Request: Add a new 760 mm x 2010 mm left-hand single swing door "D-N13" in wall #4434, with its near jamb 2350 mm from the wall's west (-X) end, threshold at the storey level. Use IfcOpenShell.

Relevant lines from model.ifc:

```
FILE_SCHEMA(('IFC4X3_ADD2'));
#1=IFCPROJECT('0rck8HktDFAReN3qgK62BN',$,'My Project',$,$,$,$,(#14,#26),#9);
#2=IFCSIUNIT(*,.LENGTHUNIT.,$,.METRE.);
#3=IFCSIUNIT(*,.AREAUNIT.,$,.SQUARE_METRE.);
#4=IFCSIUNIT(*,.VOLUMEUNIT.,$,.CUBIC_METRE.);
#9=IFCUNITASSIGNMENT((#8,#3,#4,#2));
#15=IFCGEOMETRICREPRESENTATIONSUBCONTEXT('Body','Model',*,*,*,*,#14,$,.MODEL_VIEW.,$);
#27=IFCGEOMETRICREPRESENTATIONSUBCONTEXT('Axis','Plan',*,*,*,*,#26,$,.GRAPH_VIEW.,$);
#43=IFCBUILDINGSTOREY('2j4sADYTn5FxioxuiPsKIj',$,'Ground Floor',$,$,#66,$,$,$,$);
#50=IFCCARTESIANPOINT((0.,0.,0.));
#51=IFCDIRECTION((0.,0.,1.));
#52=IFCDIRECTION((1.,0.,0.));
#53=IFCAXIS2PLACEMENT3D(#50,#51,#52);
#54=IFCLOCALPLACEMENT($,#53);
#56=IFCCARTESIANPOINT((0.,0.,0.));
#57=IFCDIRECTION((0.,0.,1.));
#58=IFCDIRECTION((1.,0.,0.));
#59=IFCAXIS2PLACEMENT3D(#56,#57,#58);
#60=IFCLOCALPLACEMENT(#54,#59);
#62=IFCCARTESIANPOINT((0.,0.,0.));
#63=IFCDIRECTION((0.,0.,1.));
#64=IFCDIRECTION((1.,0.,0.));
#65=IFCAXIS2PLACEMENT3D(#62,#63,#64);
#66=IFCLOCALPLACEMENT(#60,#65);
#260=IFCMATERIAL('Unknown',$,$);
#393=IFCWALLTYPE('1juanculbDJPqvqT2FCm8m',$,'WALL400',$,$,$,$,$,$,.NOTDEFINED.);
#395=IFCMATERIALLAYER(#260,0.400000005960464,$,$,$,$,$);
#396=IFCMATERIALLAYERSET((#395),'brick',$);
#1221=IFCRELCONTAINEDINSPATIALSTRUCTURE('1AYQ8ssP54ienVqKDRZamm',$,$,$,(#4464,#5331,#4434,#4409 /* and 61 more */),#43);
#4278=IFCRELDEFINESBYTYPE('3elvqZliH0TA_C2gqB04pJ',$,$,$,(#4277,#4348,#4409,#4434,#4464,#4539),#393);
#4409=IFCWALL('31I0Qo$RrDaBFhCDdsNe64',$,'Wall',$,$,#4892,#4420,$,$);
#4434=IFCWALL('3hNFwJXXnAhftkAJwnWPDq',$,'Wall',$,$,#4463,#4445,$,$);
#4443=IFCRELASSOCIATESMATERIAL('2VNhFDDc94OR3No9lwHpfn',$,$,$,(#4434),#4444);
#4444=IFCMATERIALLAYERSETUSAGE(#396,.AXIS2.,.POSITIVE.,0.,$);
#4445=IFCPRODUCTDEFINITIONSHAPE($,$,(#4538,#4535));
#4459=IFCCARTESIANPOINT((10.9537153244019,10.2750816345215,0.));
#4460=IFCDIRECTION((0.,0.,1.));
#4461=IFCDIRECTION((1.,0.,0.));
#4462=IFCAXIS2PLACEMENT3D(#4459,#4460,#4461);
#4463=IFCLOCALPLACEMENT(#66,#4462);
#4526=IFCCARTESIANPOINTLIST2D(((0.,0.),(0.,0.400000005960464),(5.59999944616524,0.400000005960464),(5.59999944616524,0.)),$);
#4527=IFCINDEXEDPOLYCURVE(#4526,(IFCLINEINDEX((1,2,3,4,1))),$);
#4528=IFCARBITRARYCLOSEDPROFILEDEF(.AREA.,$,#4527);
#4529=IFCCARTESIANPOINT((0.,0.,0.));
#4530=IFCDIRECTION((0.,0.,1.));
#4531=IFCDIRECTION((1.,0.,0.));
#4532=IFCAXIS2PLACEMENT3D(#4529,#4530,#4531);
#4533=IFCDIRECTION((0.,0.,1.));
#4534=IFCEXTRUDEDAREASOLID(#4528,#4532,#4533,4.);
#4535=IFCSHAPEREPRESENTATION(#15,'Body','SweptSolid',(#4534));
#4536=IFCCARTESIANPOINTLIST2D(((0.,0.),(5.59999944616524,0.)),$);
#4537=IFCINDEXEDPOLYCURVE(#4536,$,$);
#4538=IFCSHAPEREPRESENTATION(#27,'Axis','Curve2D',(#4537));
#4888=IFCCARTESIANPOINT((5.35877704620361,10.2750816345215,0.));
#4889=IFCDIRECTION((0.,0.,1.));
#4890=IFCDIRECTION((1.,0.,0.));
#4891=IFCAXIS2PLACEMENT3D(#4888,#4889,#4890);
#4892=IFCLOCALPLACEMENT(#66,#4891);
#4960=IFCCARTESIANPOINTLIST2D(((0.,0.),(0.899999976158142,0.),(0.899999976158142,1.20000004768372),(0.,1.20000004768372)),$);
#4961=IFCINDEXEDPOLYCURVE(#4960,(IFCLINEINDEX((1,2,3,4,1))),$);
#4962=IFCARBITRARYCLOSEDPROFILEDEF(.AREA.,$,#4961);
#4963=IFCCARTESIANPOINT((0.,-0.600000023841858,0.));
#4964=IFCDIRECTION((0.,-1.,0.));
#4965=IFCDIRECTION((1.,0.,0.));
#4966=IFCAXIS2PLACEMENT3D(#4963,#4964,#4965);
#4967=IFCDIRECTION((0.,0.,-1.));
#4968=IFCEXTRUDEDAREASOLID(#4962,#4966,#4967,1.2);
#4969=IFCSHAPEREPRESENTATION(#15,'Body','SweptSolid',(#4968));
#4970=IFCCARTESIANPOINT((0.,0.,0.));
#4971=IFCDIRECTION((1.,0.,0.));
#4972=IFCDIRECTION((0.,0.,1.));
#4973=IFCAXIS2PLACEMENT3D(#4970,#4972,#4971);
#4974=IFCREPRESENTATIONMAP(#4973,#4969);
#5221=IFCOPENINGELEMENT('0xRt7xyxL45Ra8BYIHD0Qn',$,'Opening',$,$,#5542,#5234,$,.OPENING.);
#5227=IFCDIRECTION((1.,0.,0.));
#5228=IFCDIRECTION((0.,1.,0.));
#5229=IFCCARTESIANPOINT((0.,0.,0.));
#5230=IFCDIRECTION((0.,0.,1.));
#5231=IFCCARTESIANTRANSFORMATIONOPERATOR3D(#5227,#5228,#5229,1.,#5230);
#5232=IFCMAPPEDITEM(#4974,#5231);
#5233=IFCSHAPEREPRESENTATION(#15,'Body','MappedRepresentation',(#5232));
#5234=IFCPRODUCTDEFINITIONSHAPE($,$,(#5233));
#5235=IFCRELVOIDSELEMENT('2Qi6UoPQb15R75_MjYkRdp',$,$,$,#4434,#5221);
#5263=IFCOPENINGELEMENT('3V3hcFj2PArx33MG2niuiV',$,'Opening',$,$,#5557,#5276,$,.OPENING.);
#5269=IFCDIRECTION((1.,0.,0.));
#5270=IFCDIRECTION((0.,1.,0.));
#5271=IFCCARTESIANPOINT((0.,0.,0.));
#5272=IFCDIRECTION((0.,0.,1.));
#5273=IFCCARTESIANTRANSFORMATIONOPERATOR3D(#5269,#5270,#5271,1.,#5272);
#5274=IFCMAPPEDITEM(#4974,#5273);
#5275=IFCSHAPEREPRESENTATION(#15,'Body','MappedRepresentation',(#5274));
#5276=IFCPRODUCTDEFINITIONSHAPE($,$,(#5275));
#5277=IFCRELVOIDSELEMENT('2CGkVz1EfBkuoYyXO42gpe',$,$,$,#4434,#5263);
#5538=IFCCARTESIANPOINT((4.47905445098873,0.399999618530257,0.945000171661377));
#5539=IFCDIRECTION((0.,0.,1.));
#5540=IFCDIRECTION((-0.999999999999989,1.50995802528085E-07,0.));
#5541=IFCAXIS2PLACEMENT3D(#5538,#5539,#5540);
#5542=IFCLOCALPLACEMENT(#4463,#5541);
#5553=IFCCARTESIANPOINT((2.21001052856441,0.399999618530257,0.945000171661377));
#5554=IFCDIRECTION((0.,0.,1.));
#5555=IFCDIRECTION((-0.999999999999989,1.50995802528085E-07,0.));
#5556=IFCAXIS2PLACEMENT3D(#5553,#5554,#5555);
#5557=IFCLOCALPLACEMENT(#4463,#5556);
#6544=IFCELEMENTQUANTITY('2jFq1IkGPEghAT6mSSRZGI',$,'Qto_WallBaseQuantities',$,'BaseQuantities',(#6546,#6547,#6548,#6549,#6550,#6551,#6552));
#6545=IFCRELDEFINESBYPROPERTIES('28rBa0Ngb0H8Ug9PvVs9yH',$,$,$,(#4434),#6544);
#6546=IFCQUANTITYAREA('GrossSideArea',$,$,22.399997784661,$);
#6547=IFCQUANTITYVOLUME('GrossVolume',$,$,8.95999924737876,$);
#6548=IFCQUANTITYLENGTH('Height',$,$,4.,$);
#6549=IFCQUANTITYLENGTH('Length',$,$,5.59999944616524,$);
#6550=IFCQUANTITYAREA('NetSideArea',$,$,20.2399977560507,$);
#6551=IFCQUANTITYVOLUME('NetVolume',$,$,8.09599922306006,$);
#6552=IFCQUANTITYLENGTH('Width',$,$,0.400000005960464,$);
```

```python
import numpy as np
import ifcopenshell
import ifcopenshell.api.feature
import ifcopenshell.api.geometry
import ifcopenshell.api.pset
import ifcopenshell.api.root
import ifcopenshell.api.spatial
import ifcopenshell.geom
import ifcopenshell.util.element
import ifcopenshell.util.placement
import ifcopenshell.util.representation
import ifcopenshell.util.shape
import ifcopenshell.util.unit

model = ifcopenshell.open("model.ifc")
unit_scale = ifcopenshell.util.unit.calculate_unit_scale(model)
area_scale = ifcopenshell.util.unit.calculate_unit_scale(model, "AREAUNIT")
volume_scale = ifcopenshell.util.unit.calculate_unit_scale(model, "VOLUMEUNIT")
settings = ifcopenshell.geom.settings()


def volume(element):
    """Net volume in cubic metres, openings subtracted."""
    shape = ifcopenshell.geom.create_shape(settings, element)
    return ifcopenshell.util.shape.get_volume(shape.geometry)


wall = model.by_guid("3hNFwJXXnAhftkAJwnWPDq")
storey = ifcopenshell.util.element.get_container(wall, ifc_class="IfcBuildingStorey")
context = ifcopenshell.util.representation.get_context(model, "Model", "Body", "MODEL_VIEW")
before = volume(wall)

width, height, from_end, sill = 0.76, 2.01, 2.35, 0.0  # metres

# The wall runs along its own X axis, and the end named is its -X end.
wall_shape = ifcopenshell.geom.create_shape(settings, wall)
x, y, z = ifcopenshell.util.shape.get_vertices(wall_shape.geometry).T
start = x.min() + from_end
face, thickness = float(y.min()), float(y.max() - y.min())
wall_matrix = ifcopenshell.util.placement.get_local_placement(wall.ObjectPlacement)
level = ifcopenshell.util.placement.get_local_placement(storey.ObjectPlacement)[2, 3]


def in_wall(x, y):
    """Placement at x, y metres in the wall's axes, at sill height."""
    matrix = wall_matrix.copy()
    matrix[:, 3] = wall_matrix @ np.array([x / unit_scale, y / unit_scale, 0.0, 1.0])
    matrix[2, 3] = level + sill / unit_scale
    return matrix


# Opening: a box that overshoots both wall faces by 50 mm.
opening = ifcopenshell.api.root.create_entity(model, ifc_class="IfcOpeningElement", predefined_type="OPENING")
box = ifcopenshell.api.geometry.add_wall_representation(
    model, context=context, length=width, height=height, thickness=thickness + 0.1
)
ifcopenshell.api.geometry.assign_representation(model, product=opening, representation=box)
ifcopenshell.api.geometry.edit_object_placement(model, product=opening, matrix=in_wall(start, face - 0.05), is_si=False)
ifcopenshell.api.feature.add_feature(model, feature=opening, element=wall)

door = ifcopenshell.api.root.create_entity(model, ifc_class="IfcDoor", name="D-N13", predefined_type="DOOR")
door.OverallWidth, door.OverallHeight = width / unit_scale, height / unit_scale
door.OperationType = "SINGLE_SWING_LEFT"
body = ifcopenshell.api.geometry.add_door_representation(
    model,
    context=context,
    overall_width=door.OverallWidth,
    overall_height=door.OverallHeight,
    operation_type="SINGLE_SWING_LEFT",
    lining_properties={"LiningDepth": thickness / unit_scale, "ThresholdDepth": thickness / unit_scale},
)
ifcopenshell.api.geometry.assign_representation(model, product=door, representation=body)
ifcopenshell.api.spatial.assign_container(model, products=[door], relating_structure=storey)
ifcopenshell.api.feature.add_filling(model, opening=opening, element=door)

# The lining spans the wall, so the door starts at the wall face.
ifcopenshell.api.geometry.edit_object_placement(model, product=door, matrix=in_wall(start, face), is_si=False)

after = volume(wall)

# Update the wall's stored quantities.
qto = model.by_id(ifcopenshell.util.element.get_pset(wall, "Qto_WallBaseQuantities", should_inherit=False)["id"])
ifcopenshell.api.pset.edit_qto(model, qto=qto, properties={
    "NetSideArea": after / thickness / area_scale,
    "NetVolume": after / volume_scale,
})

print(f"wall volume {before:.3f} -> {after:.3f} m3")

model.write("model_updated.ifc")
```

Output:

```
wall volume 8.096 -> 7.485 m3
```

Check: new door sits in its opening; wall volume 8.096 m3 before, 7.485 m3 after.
